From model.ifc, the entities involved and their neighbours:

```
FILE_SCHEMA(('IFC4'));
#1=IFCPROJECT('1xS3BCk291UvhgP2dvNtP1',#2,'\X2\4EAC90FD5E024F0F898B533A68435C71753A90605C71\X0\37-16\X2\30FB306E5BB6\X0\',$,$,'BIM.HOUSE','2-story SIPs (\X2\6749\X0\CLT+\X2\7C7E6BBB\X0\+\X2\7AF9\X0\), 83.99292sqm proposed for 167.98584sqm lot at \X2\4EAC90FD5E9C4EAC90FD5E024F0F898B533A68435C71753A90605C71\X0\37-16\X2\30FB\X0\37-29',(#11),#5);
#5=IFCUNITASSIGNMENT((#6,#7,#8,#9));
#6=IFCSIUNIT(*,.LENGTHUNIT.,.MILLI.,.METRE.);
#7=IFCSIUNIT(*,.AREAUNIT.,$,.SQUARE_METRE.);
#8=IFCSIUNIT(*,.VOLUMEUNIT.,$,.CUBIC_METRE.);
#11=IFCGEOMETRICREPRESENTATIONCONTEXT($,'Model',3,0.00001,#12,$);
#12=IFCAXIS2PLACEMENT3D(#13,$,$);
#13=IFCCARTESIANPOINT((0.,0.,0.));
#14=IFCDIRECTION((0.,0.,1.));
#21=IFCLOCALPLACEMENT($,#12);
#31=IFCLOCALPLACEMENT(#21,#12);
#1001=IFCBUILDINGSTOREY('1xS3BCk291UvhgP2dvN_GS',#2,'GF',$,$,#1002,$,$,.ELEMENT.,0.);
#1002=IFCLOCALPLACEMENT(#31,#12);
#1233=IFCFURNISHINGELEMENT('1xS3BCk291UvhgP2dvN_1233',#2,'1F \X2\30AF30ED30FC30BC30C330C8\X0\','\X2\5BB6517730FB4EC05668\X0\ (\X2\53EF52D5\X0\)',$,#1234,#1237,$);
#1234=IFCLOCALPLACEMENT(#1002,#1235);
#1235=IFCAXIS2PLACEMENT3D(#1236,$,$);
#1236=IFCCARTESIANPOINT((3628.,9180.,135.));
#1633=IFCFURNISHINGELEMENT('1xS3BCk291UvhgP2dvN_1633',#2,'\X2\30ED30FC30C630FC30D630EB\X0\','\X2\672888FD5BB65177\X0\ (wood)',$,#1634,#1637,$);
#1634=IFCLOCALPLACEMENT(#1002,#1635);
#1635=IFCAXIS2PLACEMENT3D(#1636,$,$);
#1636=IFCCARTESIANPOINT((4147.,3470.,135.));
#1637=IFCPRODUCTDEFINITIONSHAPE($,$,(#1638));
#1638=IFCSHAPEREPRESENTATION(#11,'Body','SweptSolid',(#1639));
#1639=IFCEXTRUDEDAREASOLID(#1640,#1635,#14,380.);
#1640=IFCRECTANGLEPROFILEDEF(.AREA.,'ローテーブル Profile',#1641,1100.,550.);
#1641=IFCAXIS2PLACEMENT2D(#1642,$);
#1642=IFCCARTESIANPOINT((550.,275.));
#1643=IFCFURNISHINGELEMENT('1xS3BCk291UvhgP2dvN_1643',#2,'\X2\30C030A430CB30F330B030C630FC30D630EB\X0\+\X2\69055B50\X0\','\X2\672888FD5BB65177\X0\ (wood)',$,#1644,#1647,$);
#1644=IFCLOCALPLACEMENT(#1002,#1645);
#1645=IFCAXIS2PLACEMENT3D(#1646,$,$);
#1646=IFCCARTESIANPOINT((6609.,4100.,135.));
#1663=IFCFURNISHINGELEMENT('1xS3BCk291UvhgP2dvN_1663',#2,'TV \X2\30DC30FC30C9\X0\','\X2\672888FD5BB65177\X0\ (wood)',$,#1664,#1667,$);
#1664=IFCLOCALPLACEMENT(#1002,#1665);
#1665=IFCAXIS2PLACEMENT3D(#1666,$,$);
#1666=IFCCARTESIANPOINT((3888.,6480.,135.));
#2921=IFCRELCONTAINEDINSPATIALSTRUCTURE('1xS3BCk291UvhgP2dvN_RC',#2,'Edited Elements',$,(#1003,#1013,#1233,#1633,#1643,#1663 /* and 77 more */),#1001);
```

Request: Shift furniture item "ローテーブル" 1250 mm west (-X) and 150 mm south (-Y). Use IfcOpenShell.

```python
import ifcopenshell
import ifcopenshell.api.geometry
import ifcopenshell.util.placement

model = ifcopenshell.open("model.ifc")

item = model.by_id(1633)
matrix = ifcopenshell.util.placement.get_local_placement(item.ObjectPlacement)
matrix[0, 3] -= 1250.0
matrix[1, 3] -= 150.0
ifcopenshell.api.geometry.edit_object_placement(model, product=item, matrix=matrix, is_si=False)

print(ifcopenshell.util.placement.get_local_placement(item.ObjectPlacement).round(3) + 0.0)

model.write("model_updated.ifc")
```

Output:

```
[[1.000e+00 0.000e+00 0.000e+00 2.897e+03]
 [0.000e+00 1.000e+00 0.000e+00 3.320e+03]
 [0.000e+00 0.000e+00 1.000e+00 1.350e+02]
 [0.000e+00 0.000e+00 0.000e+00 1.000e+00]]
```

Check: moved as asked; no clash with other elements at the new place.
